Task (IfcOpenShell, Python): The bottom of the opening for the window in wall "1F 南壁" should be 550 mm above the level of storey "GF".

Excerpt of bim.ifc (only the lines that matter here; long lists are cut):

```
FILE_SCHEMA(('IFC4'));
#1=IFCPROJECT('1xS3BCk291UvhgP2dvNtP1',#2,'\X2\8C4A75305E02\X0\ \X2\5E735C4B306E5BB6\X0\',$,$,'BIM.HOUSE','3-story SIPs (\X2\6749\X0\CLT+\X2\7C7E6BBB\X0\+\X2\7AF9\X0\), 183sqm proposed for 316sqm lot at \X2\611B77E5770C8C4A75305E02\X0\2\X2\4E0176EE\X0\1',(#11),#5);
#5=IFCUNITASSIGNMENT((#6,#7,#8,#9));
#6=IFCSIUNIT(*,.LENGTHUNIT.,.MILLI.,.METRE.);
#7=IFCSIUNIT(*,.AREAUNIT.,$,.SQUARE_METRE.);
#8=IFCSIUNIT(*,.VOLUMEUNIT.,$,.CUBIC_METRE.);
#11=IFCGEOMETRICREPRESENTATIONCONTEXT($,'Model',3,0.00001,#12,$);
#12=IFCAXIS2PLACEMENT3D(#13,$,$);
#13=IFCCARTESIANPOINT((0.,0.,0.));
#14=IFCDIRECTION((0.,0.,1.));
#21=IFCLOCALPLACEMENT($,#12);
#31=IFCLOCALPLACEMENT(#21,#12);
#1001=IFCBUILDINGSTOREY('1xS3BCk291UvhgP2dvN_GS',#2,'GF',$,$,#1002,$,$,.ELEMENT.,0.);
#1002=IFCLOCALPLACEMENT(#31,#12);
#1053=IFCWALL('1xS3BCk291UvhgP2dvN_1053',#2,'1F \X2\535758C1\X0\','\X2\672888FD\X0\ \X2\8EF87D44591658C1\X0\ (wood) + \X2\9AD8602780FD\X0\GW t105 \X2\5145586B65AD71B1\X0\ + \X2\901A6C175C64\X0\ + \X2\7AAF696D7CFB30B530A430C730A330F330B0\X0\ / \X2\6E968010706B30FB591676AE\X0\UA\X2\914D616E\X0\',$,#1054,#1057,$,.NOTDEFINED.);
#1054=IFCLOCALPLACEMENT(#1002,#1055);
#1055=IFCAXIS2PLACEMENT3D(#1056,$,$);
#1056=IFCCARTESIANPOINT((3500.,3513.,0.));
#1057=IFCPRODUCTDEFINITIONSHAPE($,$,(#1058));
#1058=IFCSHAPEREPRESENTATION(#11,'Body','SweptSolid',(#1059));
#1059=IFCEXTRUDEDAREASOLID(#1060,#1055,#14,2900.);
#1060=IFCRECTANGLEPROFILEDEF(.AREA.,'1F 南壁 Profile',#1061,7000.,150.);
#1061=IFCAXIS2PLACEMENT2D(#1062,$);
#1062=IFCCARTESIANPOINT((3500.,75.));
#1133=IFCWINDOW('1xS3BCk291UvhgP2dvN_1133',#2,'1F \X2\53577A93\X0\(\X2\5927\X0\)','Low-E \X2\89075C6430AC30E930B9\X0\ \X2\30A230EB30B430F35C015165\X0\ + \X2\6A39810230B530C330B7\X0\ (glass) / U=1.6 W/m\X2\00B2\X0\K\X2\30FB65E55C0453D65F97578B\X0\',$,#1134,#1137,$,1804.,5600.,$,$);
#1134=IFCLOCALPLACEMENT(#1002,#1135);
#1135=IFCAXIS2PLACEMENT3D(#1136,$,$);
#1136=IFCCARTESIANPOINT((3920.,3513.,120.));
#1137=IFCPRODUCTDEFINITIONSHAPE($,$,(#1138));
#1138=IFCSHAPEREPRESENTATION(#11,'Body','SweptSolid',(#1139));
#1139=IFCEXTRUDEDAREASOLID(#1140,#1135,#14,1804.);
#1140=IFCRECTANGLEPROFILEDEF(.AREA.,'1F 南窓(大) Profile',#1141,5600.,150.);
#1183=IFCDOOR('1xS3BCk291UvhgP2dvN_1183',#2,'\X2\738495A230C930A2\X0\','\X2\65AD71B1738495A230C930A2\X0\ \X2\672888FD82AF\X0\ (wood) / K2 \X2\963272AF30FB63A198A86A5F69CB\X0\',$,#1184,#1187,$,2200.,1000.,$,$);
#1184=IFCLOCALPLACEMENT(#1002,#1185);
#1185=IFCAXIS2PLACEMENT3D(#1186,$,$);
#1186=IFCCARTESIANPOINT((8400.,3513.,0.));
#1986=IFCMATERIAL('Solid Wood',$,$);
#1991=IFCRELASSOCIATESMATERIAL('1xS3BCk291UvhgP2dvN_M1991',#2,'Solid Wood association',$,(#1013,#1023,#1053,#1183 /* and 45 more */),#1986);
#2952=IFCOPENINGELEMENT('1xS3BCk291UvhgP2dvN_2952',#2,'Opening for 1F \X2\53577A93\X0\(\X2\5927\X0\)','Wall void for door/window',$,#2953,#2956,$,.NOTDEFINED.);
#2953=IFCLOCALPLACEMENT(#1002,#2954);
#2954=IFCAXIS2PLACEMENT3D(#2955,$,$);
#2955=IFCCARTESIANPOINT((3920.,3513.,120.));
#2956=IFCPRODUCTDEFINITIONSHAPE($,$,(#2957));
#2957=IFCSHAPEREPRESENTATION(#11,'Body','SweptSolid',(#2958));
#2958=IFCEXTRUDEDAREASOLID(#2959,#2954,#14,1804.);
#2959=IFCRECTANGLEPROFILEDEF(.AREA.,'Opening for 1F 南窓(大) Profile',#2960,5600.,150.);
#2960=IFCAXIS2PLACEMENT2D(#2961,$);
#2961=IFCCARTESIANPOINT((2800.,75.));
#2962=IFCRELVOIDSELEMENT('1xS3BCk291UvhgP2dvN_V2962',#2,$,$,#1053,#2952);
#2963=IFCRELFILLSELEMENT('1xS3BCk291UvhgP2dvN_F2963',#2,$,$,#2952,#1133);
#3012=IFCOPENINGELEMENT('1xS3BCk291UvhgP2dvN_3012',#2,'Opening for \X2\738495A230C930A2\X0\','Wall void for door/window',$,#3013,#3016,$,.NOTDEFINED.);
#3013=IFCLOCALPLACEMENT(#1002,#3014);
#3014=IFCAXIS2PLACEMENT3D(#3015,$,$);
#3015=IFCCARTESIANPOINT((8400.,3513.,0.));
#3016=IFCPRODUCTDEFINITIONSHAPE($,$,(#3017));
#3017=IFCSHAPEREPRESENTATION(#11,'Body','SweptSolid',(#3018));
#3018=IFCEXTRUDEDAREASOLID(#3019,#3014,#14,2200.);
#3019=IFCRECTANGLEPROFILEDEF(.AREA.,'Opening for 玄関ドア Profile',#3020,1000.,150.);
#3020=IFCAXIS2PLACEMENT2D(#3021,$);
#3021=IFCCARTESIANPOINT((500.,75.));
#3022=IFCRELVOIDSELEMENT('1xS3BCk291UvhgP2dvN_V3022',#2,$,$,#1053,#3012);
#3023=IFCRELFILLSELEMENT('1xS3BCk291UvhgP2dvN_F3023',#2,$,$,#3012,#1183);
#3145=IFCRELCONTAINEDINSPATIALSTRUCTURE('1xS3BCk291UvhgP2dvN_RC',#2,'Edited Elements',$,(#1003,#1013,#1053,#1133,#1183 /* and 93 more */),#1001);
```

```python
import numpy as np
import ifcopenshell
import ifcopenshell.api.geometry
import ifcopenshell.geom
import ifcopenshell.util.element
import ifcopenshell.util.placement
import ifcopenshell.util.shape
import ifcopenshell.util.unit

model = ifcopenshell.open("bim.ifc")
unit_scale = ifcopenshell.util.unit.calculate_unit_scale(model)

window = model.by_guid("1xS3BCk291UvhgP2dvN_1133")
opening = window.FillsVoids[0].RelatingOpeningElement
storey = ifcopenshell.util.element.get_container(window, ifc_class="IfcBuildingStorey")
level = ifcopenshell.util.placement.get_local_placement(storey.ObjectPlacement)[2, 3]

# The opening's origin need not be at the sill, so measure its lowest point.
shape = ifcopenshell.geom.create_shape(ifcopenshell.geom.settings(), opening)
bottom = ifcopenshell.util.shape.get_shape_bottom_elevation(shape, shape.geometry) / unit_scale
dz = level + 0.55 / unit_scale - bottom

shift = np.array([0.0, 0.0, dz])
# The window is not placed relative to its opening, so move both.
for product in (opening, window):
    matrix = ifcopenshell.util.placement.get_local_placement(product.ObjectPlacement)
    matrix[:3, 3] += shift
    ifcopenshell.api.geometry.edit_object_placement(model, product=product, matrix=matrix, is_si=False)

print(f"moved by {dz * unit_scale:+.3f} m")

model.write("bim_updated.ifc")
```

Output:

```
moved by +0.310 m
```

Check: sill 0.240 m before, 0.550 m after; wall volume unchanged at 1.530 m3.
